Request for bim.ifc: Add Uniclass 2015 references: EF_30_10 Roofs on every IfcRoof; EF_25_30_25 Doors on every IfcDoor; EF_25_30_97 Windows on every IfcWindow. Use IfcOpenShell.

First a look at what the model holds.

```python
import ifcopenshell

model = ifcopenshell.open("bim.ifc")
print(model.schema)
print("classifications:", [c.Name for c in model.by_type("IfcClassification")])
for ifc_class in ("IfcDoor", "IfcRoof", "IfcStair", "IfcWall", "IfcWindow"):
    print(ifc_class, len(model.by_type(ifc_class)))
```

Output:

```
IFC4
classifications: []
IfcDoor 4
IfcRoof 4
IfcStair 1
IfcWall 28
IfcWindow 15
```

```python
import ifcopenshell
import ifcopenshell.api.classification

model = ifcopenshell.open("bim.ifc")

system = ifcopenshell.api.classification.add_classification(model, classification="Uniclass 2015")

codes = {
    "IfcRoof": ("EF_30_10", "Roofs"),
    "IfcDoor": ("EF_25_30_25", "Doors"),
    "IfcWindow": ("EF_25_30_97", "Windows"),
}
for ifc_class, (code, name) in codes.items():
    products = model.by_type(ifc_class)
    ifcopenshell.api.classification.add_reference(
        model, products=products, classification=system, identification=code, name=name
    )
    print(code, len(products))

model.write("bim-out.ifc")
```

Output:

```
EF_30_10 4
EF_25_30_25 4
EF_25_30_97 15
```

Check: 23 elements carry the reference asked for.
